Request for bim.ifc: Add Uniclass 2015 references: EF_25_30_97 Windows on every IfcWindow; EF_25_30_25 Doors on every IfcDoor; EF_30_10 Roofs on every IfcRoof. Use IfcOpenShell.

First a look at what the model holds.

```python
import ifcopenshell

model = ifcopenshell.open("bim.ifc")
print(model.schema)
print("classifications:", [c.Name for c in model.by_type("IfcClassification")])
for ifc_class in ("IfcDoor", "IfcRoof", "IfcStair", "IfcWall", "IfcWindow"):
    print(ifc_class, len(model.by_type(ifc_class)))
```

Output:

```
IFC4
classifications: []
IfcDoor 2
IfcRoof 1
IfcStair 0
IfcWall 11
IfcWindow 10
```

```python
import ifcopenshell
import ifcopenshell.api.classification

model = ifcopenshell.open("bim.ifc")

system = ifcopenshell.api.classification.add_classification(model, classification="Uniclass 2015")

codes = {
    "IfcWindow": ("EF_25_30_97", "Windows"),
    "IfcDoor": ("EF_25_30_25", "Doors"),
    "IfcRoof": ("EF_30_10", "Roofs"),
}
for ifc_class, (code, name) in codes.items():
    products = model.by_type(ifc_class)
    ifcopenshell.api.classification.add_reference(
        model, products=products, classification=system, identification=code, name=name
    )
    print(code, len(products))

model.write("bim-out.ifc")
```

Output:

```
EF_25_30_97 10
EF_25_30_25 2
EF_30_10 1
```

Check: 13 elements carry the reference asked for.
